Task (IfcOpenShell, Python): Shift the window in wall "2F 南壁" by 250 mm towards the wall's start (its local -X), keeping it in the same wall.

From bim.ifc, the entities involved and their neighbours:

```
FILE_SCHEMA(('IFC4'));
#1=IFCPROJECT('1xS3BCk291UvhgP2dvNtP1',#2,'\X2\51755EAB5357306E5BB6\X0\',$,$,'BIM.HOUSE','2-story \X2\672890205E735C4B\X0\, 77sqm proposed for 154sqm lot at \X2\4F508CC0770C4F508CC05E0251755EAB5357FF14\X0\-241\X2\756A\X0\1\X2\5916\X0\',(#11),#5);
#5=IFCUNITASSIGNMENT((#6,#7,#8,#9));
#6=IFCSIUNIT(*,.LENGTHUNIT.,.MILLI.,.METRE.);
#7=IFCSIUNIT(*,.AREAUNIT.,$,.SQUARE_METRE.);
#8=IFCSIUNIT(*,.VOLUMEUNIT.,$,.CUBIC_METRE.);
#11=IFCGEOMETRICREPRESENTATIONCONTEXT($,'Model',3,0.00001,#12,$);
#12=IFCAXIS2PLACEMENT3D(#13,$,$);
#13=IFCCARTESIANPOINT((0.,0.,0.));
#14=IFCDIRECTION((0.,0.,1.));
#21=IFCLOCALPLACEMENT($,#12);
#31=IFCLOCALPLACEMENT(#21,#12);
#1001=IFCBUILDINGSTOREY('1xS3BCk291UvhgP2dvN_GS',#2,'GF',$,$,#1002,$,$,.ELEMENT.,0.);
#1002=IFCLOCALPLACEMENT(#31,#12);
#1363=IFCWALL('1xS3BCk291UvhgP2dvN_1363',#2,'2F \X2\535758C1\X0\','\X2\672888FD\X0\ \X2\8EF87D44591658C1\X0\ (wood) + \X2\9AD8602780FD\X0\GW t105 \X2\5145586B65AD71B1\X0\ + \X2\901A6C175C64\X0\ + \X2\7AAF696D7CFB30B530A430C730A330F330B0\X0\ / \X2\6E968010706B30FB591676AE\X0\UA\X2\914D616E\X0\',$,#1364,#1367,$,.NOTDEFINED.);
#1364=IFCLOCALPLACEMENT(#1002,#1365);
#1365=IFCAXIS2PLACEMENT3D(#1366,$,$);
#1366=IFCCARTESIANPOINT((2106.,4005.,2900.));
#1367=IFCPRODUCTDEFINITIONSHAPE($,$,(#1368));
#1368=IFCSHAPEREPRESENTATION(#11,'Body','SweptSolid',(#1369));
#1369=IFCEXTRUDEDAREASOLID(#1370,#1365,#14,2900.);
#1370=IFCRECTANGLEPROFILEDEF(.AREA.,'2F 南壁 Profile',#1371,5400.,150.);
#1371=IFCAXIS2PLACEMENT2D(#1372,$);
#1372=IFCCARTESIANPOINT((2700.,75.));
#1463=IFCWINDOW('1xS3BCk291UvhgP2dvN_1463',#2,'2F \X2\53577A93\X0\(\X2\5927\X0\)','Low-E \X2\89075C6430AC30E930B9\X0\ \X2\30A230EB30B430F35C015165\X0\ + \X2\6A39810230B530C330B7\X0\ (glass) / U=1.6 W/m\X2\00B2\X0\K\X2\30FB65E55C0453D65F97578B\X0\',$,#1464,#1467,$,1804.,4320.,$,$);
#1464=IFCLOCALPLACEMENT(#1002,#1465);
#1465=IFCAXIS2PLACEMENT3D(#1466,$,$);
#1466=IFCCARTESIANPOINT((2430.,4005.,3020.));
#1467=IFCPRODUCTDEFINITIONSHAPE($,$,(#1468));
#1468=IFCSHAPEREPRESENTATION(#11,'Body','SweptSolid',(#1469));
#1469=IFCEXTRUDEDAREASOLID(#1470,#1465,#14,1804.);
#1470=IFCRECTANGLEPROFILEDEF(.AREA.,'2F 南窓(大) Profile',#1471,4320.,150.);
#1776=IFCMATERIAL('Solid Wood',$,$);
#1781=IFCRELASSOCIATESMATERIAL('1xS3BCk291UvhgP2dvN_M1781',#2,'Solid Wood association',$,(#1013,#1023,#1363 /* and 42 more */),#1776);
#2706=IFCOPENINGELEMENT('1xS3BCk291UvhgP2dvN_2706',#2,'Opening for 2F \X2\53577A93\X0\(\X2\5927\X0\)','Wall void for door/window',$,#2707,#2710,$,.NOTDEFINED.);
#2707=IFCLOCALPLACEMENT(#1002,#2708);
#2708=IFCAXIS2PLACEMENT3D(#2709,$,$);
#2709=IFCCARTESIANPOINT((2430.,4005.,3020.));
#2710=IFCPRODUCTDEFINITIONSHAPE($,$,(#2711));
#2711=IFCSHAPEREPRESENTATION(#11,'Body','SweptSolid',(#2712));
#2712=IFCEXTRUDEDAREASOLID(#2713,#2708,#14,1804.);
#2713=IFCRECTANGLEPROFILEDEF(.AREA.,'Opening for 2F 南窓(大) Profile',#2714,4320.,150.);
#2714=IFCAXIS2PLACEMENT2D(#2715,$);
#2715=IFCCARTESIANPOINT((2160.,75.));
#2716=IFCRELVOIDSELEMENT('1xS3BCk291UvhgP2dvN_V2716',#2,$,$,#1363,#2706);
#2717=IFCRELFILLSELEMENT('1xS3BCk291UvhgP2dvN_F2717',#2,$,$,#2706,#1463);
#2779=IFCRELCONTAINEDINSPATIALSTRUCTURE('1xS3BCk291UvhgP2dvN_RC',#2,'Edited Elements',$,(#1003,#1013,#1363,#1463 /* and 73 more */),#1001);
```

```python
import ifcopenshell
import ifcopenshell.api.geometry
import ifcopenshell.util.placement
import ifcopenshell.util.unit

model = ifcopenshell.open("bim.ifc")
unit_scale = ifcopenshell.util.unit.calculate_unit_scale(model)

window = model.by_id(1463)
opening = window.FillsVoids[0].RelatingOpeningElement
wall = opening.VoidsElements[0].RelatingBuildingElement

wall_matrix = ifcopenshell.util.placement.get_local_placement(wall.ObjectPlacement)
shift = wall_matrix[:3, 0] * -0.25 / unit_scale
before = ifcopenshell.util.placement.get_local_placement(window.ObjectPlacement)[:3, 3].copy()

# The window is not placed relative to its opening, so move both.
for product in (opening, window):
    matrix = ifcopenshell.util.placement.get_local_placement(product.ObjectPlacement)
    matrix[:3, 3] += shift
    ifcopenshell.api.geometry.edit_object_placement(model, product=product, matrix=matrix, is_si=False)

after = ifcopenshell.util.placement.get_local_placement(window.ObjectPlacement)[:3, 3]
print("window moved by", (after - before).round(3) + 0.0)

model.write("bim-out.ifc")
```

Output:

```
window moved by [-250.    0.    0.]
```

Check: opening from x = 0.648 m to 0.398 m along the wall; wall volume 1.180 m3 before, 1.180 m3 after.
